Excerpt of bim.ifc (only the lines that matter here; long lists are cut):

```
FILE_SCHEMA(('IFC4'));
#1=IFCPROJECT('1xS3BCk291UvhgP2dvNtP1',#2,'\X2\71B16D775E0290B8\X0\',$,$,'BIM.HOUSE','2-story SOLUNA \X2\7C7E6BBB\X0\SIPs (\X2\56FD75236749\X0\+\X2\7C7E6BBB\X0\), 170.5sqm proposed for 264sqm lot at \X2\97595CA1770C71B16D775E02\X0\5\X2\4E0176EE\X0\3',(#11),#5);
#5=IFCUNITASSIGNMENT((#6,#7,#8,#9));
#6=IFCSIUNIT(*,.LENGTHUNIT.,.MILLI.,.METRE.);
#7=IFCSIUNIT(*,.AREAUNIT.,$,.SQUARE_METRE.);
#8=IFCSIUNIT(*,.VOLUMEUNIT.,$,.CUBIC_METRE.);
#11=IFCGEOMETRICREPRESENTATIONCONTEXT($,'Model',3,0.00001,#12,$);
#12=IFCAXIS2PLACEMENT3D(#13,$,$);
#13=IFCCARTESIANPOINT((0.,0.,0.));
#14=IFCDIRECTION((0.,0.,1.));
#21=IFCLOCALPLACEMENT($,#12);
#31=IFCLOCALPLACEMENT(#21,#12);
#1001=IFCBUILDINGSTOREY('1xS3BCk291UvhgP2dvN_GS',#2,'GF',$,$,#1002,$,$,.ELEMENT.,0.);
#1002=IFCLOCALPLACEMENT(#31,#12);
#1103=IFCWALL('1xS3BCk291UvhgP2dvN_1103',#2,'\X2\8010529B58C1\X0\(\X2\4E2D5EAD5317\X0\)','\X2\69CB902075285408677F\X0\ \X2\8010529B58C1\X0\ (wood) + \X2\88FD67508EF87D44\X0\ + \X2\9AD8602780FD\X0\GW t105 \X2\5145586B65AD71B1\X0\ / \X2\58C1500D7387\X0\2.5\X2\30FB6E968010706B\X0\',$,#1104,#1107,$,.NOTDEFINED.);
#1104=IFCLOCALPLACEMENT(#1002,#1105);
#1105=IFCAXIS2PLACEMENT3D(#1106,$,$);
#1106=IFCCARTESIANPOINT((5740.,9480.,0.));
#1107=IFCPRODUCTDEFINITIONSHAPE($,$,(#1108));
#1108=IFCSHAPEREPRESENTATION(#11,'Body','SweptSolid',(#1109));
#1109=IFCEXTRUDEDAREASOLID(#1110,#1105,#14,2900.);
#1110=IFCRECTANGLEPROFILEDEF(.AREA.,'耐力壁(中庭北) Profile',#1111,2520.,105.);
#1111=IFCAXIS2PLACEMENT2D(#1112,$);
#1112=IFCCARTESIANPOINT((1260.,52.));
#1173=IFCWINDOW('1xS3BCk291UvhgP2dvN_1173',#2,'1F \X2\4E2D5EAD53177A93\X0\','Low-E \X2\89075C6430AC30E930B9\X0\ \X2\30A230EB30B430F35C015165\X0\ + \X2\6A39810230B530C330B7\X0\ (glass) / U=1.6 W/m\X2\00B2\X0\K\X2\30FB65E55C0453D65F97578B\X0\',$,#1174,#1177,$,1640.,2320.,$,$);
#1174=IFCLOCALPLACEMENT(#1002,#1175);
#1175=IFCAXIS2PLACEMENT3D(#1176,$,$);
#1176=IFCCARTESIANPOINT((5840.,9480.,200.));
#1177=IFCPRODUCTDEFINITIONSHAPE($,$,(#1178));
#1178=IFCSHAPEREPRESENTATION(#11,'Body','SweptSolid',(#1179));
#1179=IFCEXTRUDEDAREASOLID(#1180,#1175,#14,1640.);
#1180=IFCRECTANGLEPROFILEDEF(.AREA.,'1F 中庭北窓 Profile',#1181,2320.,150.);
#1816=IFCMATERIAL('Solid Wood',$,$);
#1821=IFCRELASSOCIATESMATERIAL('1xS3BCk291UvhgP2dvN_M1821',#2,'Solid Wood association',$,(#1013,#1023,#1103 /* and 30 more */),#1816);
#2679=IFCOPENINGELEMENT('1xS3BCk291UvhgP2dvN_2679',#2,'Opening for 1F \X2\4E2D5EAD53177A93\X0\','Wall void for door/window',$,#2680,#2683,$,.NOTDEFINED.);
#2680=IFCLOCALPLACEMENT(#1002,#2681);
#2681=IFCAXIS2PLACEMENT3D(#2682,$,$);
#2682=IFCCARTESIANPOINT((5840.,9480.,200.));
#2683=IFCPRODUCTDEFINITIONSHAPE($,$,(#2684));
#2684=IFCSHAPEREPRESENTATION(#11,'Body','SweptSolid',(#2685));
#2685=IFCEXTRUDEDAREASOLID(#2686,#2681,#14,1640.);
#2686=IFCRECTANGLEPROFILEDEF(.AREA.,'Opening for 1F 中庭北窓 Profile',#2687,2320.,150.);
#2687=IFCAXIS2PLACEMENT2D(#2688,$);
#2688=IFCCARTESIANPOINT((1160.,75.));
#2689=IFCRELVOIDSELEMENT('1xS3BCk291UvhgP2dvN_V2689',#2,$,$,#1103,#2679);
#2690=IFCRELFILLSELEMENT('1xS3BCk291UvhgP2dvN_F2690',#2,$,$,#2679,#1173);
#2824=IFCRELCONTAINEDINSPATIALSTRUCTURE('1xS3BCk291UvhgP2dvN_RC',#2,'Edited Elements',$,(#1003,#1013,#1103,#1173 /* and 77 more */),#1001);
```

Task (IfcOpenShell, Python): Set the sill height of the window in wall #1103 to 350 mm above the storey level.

```python
import numpy as np
import ifcopenshell
import ifcopenshell.api.geometry
import ifcopenshell.geom
import ifcopenshell.util.element
import ifcopenshell.util.placement
import ifcopenshell.util.shape
import ifcopenshell.util.unit

model = ifcopenshell.open("bim.ifc")
unit_scale = ifcopenshell.util.unit.calculate_unit_scale(model)

window = model.by_guid("1xS3BCk291UvhgP2dvN_1173")
opening = window.FillsVoids[0].RelatingOpeningElement
storey = ifcopenshell.util.element.get_container(window, ifc_class="IfcBuildingStorey")
level = ifcopenshell.util.placement.get_local_placement(storey.ObjectPlacement)[2, 3]

# The opening's origin need not be at the sill, so measure its lowest point.
shape = ifcopenshell.geom.create_shape(ifcopenshell.geom.settings(), opening)
bottom = ifcopenshell.util.shape.get_shape_bottom_elevation(shape, shape.geometry) / unit_scale
dz = level + 350.0 - bottom

shift = np.array([0.0, 0.0, dz])
# The window is not placed relative to its opening, so move both.
for product in (opening, window):
    matrix = ifcopenshell.util.placement.get_local_placement(product.ObjectPlacement)
    matrix[:3, 3] += shift
    ifcopenshell.api.geometry.edit_object_placement(model, product=product, matrix=matrix, is_si=False)

print(f"moved by {dz * unit_scale:+.3f} m")

model.write("bim_rev.ifc")
```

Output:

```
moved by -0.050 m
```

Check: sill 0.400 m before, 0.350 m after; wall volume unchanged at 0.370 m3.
